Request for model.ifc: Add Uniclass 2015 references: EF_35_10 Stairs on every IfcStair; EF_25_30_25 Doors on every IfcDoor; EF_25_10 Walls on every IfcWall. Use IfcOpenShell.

First a look at what the model holds.

```python
import ifcopenshell

model = ifcopenshell.open("model.ifc")
print(model.schema)
print("classifications:", [c.Name for c in model.by_type("IfcClassification")])
for ifc_class in ("IfcDoor", "IfcRoof", "IfcStair", "IfcWall", "IfcWindow"):
    print(ifc_class, len(model.by_type(ifc_class)))
```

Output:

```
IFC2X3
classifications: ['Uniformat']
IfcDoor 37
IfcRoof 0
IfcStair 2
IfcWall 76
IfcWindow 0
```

```python
import ifcopenshell
import ifcopenshell.api.classification

model = ifcopenshell.open("model.ifc")

# IFC2X3 requires Source and Edition and has no link from the project to the system.
system = model.create_entity("IfcClassification", Source="NBS", Edition="2015", Name="Uniclass 2015")

codes = {
    "IfcStair": ("EF_35_10", "Stairs"),
    "IfcDoor": ("EF_25_30_25", "Doors"),
    "IfcWall": ("EF_25_10", "Walls"),
}
for ifc_class, (code, name) in codes.items():
    products = model.by_type(ifc_class)
    ifcopenshell.api.classification.add_reference(
        model, products=products, classification=system, identification=code, name=name
    )
    print(code, len(products))

model.write("model-out.ifc")
```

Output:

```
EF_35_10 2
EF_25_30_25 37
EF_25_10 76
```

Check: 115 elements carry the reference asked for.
